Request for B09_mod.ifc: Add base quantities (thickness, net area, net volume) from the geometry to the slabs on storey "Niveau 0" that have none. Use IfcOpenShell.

First a look at what the model holds.

```python
import ifcopenshell
import ifcopenshell.util.element
import ifcopenshell.util.unit

model = ifcopenshell.open("B09_mod.ifc")
print(model.schema)
for unit_type in ("LENGTHUNIT", "AREAUNIT", "VOLUMEUNIT"):
    print(unit_type, ifcopenshell.util.unit.calculate_unit_scale(model, unit_type))
storey = next(s for s in model.by_type("IfcBuildingStorey") if s.Name == "Niveau 0")
slabs = [e for e in ifcopenshell.util.element.get_decomposition(storey) if e.is_a("IfcSlab")]
for e in sorted(slabs, key=lambda e: e.id()):
    print(e.id(), e.is_a(), e.Name, list(ifcopenshell.util.element.get_psets(e, qtos_only=True)), sep=" | ")
```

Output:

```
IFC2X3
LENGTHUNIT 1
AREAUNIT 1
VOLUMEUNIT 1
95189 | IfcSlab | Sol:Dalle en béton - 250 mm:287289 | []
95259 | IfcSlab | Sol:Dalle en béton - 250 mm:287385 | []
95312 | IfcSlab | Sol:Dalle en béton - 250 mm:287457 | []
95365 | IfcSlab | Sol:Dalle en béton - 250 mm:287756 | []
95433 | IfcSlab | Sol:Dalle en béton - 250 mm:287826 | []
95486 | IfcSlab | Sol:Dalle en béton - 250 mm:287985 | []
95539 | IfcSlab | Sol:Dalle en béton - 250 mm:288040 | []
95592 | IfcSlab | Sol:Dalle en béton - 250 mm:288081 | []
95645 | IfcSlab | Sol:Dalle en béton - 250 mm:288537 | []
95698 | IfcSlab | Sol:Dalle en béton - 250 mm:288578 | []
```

```python
import ifcopenshell
import ifcopenshell.api.pset
import ifcopenshell.geom
import ifcopenshell.util.element
import ifcopenshell.util.shape
import ifcopenshell.util.unit

model = ifcopenshell.open("B09_mod.ifc")
unit_scale = ifcopenshell.util.unit.calculate_unit_scale(model)
area_scale = ifcopenshell.util.unit.calculate_unit_scale(model, "AREAUNIT")
volume_scale = ifcopenshell.util.unit.calculate_unit_scale(model, "VOLUMEUNIT")
settings = ifcopenshell.geom.settings()

storey = next(s for s in model.by_type("IfcBuildingStorey") if s.Name == "Niveau 0")
slabs = [e for e in ifcopenshell.util.element.get_decomposition(storey) if e.is_a("IfcSlab")]

for e in sorted(slabs, key=lambda e: e.id()):
    if ifcopenshell.util.element.get_psets(e, qtos_only=True, should_inherit=False):
        continue
    # Geometry comes back in metres, in the element's own axes.
    shape = ifcopenshell.geom.create_shape(settings, e)
    values = {
        "Width": ifcopenshell.util.shape.get_z(shape.geometry) / unit_scale,
        "NetArea": ifcopenshell.util.shape.get_footprint_area(shape.geometry) / area_scale,
        "NetVolume": ifcopenshell.util.shape.get_volume(shape.geometry) / volume_scale,
    }
    qto = ifcopenshell.api.pset.add_qto(model, product=e, name="BaseQuantities")
    ifcopenshell.api.pset.edit_qto(model, qto=qto, properties=values)
    print(e.id(), {k: round(v, 3) for k, v in values.items()})

model.write("B09_mod_updated.ifc")
```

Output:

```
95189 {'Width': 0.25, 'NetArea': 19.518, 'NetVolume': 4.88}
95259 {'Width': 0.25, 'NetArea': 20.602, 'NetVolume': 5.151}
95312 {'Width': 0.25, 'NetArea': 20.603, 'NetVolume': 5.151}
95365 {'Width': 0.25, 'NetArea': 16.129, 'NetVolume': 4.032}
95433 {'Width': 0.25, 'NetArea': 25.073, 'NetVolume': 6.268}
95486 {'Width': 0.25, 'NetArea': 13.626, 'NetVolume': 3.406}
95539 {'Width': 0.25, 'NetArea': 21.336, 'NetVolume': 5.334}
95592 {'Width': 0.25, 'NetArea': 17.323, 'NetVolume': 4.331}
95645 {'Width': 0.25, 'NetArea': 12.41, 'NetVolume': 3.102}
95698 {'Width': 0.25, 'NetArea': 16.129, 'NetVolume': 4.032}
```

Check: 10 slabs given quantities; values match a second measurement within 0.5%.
